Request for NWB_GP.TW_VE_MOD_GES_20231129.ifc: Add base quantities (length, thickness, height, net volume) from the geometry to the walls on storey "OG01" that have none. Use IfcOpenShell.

First a look at what the model holds.

```python
import ifcopenshell
import ifcopenshell.util.element
import ifcopenshell.util.unit

model = ifcopenshell.open("NWB_GP.TW_VE_MOD_GES_20231129.ifc")
print(model.schema)
for unit_type in ("LENGTHUNIT", "AREAUNIT", "VOLUMEUNIT"):
    print(unit_type, ifcopenshell.util.unit.calculate_unit_scale(model, unit_type))
storey = next(s for s in model.by_type("IfcBuildingStorey") if s.Name == "OG01")
walls = [e for e in ifcopenshell.util.element.get_decomposition(storey) if e.is_a("IfcWall")]
for e in sorted(walls, key=lambda e: e.id()):
    print(e.id(), e.is_a(), e.Name, list(ifcopenshell.util.element.get_psets(e, qtos_only=True)), sep=" | ")
```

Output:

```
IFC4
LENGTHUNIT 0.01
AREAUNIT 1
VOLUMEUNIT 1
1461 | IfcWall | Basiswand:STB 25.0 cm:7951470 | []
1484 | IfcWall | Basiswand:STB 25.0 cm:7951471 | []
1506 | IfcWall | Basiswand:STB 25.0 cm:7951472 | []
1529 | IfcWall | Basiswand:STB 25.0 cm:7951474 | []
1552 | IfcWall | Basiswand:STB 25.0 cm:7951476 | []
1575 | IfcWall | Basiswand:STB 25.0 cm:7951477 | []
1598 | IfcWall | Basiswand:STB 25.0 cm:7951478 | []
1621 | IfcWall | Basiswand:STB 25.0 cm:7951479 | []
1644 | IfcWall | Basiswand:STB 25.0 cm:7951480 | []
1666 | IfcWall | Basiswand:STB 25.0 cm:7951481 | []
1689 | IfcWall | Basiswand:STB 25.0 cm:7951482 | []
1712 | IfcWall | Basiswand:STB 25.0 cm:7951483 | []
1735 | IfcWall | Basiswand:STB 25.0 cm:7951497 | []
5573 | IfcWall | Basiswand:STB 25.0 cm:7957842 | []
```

```python
import ifcopenshell
import ifcopenshell.api.pset
import ifcopenshell.geom
import ifcopenshell.util.element
import ifcopenshell.util.shape
import ifcopenshell.util.unit

model = ifcopenshell.open("NWB_GP.TW_VE_MOD_GES_20231129.ifc")
unit_scale = ifcopenshell.util.unit.calculate_unit_scale(model)
volume_scale = ifcopenshell.util.unit.calculate_unit_scale(model, "VOLUMEUNIT")
settings = ifcopenshell.geom.settings()

storey = next(s for s in model.by_type("IfcBuildingStorey") if s.Name == "OG01")
walls = [e for e in ifcopenshell.util.element.get_decomposition(storey) if e.is_a("IfcWall")]

for e in sorted(walls, key=lambda e: e.id()):
    if ifcopenshell.util.element.get_psets(e, qtos_only=True, should_inherit=False):
        continue
    # Geometry comes back in metres, in the element's own axes.
    shape = ifcopenshell.geom.create_shape(settings, e)
    values = {
        "Length": ifcopenshell.util.shape.get_x(shape.geometry) / unit_scale,
        "Width": ifcopenshell.util.shape.get_y(shape.geometry) / unit_scale,
        "Height": ifcopenshell.util.shape.get_z(shape.geometry) / unit_scale,
        "NetVolume": ifcopenshell.util.shape.get_volume(shape.geometry) / volume_scale,
    }
    qto = ifcopenshell.api.pset.add_qto(model, product=e, name="Qto_WallBaseQuantities")
    ifcopenshell.api.pset.edit_qto(model, qto=qto, properties=values)
    print(e.id(), {k: round(v, 3) for k, v in values.items()})

model.write("NWB_GP.TW_VE_MOD_GES_20231129_rev.ifc")
```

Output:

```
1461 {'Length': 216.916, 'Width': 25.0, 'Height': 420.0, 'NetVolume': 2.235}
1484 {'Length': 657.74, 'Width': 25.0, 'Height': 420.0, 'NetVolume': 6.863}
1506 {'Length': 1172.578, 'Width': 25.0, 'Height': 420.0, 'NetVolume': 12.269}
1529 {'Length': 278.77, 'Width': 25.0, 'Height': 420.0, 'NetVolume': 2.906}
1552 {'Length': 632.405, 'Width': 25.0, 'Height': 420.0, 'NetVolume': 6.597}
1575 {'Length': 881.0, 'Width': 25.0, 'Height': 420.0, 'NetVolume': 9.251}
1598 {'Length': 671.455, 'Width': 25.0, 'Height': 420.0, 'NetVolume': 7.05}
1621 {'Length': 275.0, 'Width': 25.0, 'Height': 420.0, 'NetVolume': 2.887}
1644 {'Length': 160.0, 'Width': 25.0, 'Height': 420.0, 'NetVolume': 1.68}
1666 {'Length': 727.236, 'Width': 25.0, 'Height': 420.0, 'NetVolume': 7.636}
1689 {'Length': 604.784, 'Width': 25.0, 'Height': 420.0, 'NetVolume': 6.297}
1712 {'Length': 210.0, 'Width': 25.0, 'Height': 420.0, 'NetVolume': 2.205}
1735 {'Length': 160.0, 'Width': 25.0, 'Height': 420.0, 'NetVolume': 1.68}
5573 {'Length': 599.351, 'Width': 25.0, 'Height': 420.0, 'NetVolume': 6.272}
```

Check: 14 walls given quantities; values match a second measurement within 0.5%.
